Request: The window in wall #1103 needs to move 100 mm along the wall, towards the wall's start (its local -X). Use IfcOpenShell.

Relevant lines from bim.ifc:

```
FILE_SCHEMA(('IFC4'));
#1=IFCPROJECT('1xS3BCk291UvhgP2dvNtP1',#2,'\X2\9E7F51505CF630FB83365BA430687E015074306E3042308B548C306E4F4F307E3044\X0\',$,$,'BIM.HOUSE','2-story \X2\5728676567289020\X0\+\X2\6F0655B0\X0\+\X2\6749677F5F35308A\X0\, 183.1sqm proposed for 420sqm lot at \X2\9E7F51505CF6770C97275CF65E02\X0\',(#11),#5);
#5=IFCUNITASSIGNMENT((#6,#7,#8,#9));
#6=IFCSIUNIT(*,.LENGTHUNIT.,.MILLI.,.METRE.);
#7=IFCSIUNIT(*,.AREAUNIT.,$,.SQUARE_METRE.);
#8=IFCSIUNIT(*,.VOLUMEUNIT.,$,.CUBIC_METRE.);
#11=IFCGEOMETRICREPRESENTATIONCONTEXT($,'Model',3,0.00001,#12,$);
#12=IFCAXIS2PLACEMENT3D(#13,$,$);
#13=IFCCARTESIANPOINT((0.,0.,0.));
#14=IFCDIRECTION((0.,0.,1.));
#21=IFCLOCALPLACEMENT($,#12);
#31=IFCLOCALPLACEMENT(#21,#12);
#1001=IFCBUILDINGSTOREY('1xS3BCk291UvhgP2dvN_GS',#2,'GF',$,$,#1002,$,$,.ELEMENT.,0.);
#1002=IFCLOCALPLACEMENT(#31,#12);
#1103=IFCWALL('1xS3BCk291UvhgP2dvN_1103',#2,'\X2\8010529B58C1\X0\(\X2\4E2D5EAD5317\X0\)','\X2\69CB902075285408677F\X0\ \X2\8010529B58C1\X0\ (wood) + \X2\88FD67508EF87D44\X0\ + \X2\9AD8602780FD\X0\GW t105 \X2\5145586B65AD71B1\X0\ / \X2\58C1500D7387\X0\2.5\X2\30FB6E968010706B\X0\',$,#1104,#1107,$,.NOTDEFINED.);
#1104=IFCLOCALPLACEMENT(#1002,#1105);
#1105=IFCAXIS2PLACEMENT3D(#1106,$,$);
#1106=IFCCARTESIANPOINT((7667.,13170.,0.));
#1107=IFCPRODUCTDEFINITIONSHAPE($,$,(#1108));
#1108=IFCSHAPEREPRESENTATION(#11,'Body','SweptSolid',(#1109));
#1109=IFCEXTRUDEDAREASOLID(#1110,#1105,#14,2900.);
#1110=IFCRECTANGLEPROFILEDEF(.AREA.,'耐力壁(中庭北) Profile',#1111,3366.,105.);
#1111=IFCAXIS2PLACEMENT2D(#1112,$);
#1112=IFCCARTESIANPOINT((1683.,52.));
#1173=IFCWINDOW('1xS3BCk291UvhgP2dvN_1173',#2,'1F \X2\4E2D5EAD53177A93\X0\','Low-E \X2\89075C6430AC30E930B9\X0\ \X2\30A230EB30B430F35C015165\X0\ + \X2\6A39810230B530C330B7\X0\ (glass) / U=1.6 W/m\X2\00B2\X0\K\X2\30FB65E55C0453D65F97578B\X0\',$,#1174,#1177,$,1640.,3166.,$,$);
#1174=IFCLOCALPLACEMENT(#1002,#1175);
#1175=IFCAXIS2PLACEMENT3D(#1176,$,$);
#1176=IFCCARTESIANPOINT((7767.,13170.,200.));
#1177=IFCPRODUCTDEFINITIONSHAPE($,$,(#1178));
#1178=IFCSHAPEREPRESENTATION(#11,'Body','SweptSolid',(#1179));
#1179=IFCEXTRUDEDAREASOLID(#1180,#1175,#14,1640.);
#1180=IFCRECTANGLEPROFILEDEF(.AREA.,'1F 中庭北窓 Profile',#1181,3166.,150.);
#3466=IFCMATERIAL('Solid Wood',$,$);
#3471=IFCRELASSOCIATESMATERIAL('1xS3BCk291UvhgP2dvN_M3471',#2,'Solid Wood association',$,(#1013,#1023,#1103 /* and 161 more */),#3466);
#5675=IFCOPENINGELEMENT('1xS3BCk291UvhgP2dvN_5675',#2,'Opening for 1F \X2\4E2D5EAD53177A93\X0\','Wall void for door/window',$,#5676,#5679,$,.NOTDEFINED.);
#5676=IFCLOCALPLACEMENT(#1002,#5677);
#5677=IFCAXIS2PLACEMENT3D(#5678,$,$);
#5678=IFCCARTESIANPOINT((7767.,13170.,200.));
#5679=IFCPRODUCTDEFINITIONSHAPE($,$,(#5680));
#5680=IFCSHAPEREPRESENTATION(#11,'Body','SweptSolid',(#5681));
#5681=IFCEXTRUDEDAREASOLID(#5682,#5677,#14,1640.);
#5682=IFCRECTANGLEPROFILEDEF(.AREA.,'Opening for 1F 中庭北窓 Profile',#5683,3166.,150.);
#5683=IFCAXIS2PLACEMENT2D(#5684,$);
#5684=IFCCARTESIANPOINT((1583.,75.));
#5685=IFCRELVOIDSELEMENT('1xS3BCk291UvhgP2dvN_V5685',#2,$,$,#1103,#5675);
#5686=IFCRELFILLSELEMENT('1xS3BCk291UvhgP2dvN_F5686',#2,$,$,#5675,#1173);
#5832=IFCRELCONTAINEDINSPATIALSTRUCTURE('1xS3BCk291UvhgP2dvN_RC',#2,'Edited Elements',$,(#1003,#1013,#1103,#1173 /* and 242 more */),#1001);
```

```python
import ifcopenshell
import ifcopenshell.api.geometry
import ifcopenshell.util.placement
import ifcopenshell.util.unit

model = ifcopenshell.open("bim.ifc")
unit_scale = ifcopenshell.util.unit.calculate_unit_scale(model)

window = model.by_guid("1xS3BCk291UvhgP2dvN_1173")
opening = window.FillsVoids[0].RelatingOpeningElement
wall = opening.VoidsElements[0].RelatingBuildingElement

wall_matrix = ifcopenshell.util.placement.get_local_placement(wall.ObjectPlacement)
shift = wall_matrix[:3, 0] * -0.1 / unit_scale
before = ifcopenshell.util.placement.get_local_placement(window.ObjectPlacement)[:3, 3].copy()

# The window is not placed relative to its opening, so move both.
for product in (opening, window):
    matrix = ifcopenshell.util.placement.get_local_placement(product.ObjectPlacement)
    matrix[:3, 3] += shift
    ifcopenshell.api.geometry.edit_object_placement(model, product=product, matrix=matrix, is_si=False)

after = ifcopenshell.util.placement.get_local_placement(window.ObjectPlacement)[:3, 3]
print("window moved by", (after - before).round(3) + 0.0)

model.write("bim-out.ifc")
```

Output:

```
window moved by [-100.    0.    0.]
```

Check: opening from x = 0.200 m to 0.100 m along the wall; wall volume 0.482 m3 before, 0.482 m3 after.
